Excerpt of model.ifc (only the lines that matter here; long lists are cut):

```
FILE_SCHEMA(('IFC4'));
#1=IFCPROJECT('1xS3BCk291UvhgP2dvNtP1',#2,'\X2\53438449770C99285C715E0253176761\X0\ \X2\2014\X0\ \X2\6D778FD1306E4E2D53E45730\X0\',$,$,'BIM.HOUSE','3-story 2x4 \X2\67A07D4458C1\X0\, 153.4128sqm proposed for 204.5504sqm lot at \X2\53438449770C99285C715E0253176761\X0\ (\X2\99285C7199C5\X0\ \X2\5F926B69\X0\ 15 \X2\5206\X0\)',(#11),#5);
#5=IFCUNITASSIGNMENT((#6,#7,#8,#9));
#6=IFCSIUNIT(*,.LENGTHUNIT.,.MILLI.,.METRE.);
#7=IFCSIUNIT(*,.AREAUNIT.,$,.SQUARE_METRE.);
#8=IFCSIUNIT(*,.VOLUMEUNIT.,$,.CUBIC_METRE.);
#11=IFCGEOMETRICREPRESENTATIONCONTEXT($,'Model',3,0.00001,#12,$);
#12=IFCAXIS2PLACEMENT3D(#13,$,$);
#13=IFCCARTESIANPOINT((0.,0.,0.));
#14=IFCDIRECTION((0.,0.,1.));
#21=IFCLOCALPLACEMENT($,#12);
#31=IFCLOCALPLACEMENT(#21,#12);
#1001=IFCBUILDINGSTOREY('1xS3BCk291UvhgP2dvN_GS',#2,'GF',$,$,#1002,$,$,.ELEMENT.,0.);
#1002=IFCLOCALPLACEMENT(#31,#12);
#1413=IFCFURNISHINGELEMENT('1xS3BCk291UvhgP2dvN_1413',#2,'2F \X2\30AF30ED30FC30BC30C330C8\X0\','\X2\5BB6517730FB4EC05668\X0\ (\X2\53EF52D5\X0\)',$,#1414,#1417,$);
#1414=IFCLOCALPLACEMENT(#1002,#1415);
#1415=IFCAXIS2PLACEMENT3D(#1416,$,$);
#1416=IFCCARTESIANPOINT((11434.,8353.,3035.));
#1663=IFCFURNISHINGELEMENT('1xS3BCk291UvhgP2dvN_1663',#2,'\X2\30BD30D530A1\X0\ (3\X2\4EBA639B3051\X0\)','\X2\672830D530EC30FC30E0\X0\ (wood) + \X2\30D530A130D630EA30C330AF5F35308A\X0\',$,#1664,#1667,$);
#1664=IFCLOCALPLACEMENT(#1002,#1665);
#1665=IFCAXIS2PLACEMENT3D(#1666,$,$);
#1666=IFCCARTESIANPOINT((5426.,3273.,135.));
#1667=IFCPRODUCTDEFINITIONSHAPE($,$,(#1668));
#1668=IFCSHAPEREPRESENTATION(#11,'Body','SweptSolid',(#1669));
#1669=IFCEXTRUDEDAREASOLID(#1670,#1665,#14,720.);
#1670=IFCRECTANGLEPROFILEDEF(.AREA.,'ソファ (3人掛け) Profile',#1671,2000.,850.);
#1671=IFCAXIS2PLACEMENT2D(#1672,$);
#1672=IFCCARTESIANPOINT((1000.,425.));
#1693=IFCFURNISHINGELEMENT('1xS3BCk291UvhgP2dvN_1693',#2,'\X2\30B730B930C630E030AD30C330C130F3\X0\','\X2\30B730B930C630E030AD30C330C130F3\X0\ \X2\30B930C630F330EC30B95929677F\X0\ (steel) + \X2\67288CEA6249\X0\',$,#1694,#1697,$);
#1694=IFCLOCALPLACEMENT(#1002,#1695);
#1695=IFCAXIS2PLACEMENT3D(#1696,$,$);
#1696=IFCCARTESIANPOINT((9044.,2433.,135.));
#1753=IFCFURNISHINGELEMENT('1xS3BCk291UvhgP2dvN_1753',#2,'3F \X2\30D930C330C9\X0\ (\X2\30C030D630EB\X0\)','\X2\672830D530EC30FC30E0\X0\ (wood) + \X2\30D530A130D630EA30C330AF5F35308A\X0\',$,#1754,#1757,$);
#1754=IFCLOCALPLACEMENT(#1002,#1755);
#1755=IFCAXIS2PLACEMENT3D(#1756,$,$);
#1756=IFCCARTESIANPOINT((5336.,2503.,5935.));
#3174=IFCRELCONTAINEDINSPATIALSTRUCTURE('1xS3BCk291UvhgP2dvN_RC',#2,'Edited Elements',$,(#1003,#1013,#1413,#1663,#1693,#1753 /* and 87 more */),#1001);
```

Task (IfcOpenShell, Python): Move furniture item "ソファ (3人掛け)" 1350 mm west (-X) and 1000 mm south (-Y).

```python
import ifcopenshell
import ifcopenshell.api.geometry
import ifcopenshell.util.placement

model = ifcopenshell.open("model.ifc")

item = model.by_guid("1xS3BCk291UvhgP2dvN_1663")
matrix = ifcopenshell.util.placement.get_local_placement(item.ObjectPlacement)
matrix[0, 3] -= 1350.0
matrix[1, 3] -= 1000.0
ifcopenshell.api.geometry.edit_object_placement(model, product=item, matrix=matrix, is_si=False)

print(ifcopenshell.util.placement.get_local_placement(item.ObjectPlacement).round(3) + 0.0)

model.write("model_rev.ifc")
```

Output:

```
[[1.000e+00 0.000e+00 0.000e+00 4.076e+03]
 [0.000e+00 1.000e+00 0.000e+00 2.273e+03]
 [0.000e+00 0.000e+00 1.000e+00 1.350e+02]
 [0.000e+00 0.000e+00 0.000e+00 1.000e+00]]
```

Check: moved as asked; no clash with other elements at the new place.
